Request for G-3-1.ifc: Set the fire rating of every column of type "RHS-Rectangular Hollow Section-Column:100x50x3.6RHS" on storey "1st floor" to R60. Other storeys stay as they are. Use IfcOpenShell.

First a look at what the model holds.

```python
import ifcopenshell
import ifcopenshell.util.element

model = ifcopenshell.open("G-3-1.ifc")
print(model.schema)
storey = next(s for s in model.by_type("IfcBuildingStorey") if s.Name == "1st floor")
columns = [e for e in ifcopenshell.util.element.get_decomposition(storey) if e.is_a("IfcColumn")]
seen = {}
for e in columns:
    element_type = ifcopenshell.util.element.get_type(e)
    key = (element_type.Name if element_type != e and element_type else None, ifcopenshell.util.element.get_pset(e, "Pset_ColumnCommon", "FireRating"))
    seen[key] = seen.get(key, 0) + 1
for (name, value), count in sorted(seen.items(), key=str):
    print(count, "x", name, "|", value)
```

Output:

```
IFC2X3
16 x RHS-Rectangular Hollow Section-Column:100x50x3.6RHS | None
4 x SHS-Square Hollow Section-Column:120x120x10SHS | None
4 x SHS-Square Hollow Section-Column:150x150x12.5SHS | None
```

```python
import ifcopenshell
import ifcopenshell.api.pset
import ifcopenshell.util.element

model = ifcopenshell.open("G-3-1.ifc")

storey = next(s for s in model.by_type("IfcBuildingStorey") if s.Name == "1st floor")
columns = [e for e in ifcopenshell.util.element.get_decomposition(storey) if e.is_a("IfcColumn")]

count = 0
for e in columns:
    element_type = ifcopenshell.util.element.get_type(e)
    if element_type in (None, e) or element_type.Name != "RHS-Rectangular Hollow Section-Column:100x50x3.6RHS":
        continue
    # add_pset returns the element's existing set when there is one.
    pset = ifcopenshell.api.pset.add_pset(model, product=e, name="Pset_ColumnCommon")
    ifcopenshell.api.pset.edit_pset(model, pset=pset, properties={"FireRating": "R60"})
    count += 1

print(count, "columns updated")

model.write("G-3-1_updated.ifc")
```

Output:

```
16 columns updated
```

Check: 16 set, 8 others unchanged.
